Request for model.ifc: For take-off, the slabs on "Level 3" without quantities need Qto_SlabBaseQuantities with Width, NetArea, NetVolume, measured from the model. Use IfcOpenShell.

First a look at what the model holds.

```python
import ifcopenshell
import ifcopenshell.util.element
import ifcopenshell.util.unit

model = ifcopenshell.open("model.ifc")
print(model.schema)
for unit_type in ("LENGTHUNIT", "AREAUNIT", "VOLUMEUNIT"):
    print(unit_type, ifcopenshell.util.unit.calculate_unit_scale(model, unit_type))
storey = next(s for s in model.by_type("IfcBuildingStorey") if s.Name == "Level 3")
slabs = [e for e in ifcopenshell.util.element.get_decomposition(storey) if e.is_a("IfcSlab")]
for e in sorted(slabs, key=lambda e: e.id()):
    print(e.id(), e.is_a(), e.Name, list(ifcopenshell.util.element.get_psets(e, qtos_only=True)), sep=" | ")
```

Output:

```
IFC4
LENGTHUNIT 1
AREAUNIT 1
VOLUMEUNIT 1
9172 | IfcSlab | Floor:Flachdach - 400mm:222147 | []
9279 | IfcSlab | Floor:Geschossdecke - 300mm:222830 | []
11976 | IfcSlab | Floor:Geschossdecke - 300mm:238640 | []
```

```python
import ifcopenshell
import ifcopenshell.api.pset
import ifcopenshell.geom
import ifcopenshell.util.element
import ifcopenshell.util.shape
import ifcopenshell.util.unit

model = ifcopenshell.open("model.ifc")
unit_scale = ifcopenshell.util.unit.calculate_unit_scale(model)
area_scale = ifcopenshell.util.unit.calculate_unit_scale(model, "AREAUNIT")
volume_scale = ifcopenshell.util.unit.calculate_unit_scale(model, "VOLUMEUNIT")
settings = ifcopenshell.geom.settings()

storey = next(s for s in model.by_type("IfcBuildingStorey") if s.Name == "Level 3")
slabs = [e for e in ifcopenshell.util.element.get_decomposition(storey) if e.is_a("IfcSlab")]

for e in sorted(slabs, key=lambda e: e.id()):
    if ifcopenshell.util.element.get_psets(e, qtos_only=True, should_inherit=False):
        continue
    # Geometry comes back in metres, in the element's own axes.
    shape = ifcopenshell.geom.create_shape(settings, e)
    values = {
        "Width": ifcopenshell.util.shape.get_z(shape.geometry) / unit_scale,
        "NetArea": ifcopenshell.util.shape.get_footprint_area(shape.geometry) / area_scale,
        "NetVolume": ifcopenshell.util.shape.get_volume(shape.geometry) / volume_scale,
    }
    qto = ifcopenshell.api.pset.add_qto(model, product=e, name="Qto_SlabBaseQuantities")
    ifcopenshell.api.pset.edit_qto(model, qto=qto, properties=values)
    print(e.id(), {k: round(v, 3) for k, v in values.items()})

model.write("model_rev.ifc")
```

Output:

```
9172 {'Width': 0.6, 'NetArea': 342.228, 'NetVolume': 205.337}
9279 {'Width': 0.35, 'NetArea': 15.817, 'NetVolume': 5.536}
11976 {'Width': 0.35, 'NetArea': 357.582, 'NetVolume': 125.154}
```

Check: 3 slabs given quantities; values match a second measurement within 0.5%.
